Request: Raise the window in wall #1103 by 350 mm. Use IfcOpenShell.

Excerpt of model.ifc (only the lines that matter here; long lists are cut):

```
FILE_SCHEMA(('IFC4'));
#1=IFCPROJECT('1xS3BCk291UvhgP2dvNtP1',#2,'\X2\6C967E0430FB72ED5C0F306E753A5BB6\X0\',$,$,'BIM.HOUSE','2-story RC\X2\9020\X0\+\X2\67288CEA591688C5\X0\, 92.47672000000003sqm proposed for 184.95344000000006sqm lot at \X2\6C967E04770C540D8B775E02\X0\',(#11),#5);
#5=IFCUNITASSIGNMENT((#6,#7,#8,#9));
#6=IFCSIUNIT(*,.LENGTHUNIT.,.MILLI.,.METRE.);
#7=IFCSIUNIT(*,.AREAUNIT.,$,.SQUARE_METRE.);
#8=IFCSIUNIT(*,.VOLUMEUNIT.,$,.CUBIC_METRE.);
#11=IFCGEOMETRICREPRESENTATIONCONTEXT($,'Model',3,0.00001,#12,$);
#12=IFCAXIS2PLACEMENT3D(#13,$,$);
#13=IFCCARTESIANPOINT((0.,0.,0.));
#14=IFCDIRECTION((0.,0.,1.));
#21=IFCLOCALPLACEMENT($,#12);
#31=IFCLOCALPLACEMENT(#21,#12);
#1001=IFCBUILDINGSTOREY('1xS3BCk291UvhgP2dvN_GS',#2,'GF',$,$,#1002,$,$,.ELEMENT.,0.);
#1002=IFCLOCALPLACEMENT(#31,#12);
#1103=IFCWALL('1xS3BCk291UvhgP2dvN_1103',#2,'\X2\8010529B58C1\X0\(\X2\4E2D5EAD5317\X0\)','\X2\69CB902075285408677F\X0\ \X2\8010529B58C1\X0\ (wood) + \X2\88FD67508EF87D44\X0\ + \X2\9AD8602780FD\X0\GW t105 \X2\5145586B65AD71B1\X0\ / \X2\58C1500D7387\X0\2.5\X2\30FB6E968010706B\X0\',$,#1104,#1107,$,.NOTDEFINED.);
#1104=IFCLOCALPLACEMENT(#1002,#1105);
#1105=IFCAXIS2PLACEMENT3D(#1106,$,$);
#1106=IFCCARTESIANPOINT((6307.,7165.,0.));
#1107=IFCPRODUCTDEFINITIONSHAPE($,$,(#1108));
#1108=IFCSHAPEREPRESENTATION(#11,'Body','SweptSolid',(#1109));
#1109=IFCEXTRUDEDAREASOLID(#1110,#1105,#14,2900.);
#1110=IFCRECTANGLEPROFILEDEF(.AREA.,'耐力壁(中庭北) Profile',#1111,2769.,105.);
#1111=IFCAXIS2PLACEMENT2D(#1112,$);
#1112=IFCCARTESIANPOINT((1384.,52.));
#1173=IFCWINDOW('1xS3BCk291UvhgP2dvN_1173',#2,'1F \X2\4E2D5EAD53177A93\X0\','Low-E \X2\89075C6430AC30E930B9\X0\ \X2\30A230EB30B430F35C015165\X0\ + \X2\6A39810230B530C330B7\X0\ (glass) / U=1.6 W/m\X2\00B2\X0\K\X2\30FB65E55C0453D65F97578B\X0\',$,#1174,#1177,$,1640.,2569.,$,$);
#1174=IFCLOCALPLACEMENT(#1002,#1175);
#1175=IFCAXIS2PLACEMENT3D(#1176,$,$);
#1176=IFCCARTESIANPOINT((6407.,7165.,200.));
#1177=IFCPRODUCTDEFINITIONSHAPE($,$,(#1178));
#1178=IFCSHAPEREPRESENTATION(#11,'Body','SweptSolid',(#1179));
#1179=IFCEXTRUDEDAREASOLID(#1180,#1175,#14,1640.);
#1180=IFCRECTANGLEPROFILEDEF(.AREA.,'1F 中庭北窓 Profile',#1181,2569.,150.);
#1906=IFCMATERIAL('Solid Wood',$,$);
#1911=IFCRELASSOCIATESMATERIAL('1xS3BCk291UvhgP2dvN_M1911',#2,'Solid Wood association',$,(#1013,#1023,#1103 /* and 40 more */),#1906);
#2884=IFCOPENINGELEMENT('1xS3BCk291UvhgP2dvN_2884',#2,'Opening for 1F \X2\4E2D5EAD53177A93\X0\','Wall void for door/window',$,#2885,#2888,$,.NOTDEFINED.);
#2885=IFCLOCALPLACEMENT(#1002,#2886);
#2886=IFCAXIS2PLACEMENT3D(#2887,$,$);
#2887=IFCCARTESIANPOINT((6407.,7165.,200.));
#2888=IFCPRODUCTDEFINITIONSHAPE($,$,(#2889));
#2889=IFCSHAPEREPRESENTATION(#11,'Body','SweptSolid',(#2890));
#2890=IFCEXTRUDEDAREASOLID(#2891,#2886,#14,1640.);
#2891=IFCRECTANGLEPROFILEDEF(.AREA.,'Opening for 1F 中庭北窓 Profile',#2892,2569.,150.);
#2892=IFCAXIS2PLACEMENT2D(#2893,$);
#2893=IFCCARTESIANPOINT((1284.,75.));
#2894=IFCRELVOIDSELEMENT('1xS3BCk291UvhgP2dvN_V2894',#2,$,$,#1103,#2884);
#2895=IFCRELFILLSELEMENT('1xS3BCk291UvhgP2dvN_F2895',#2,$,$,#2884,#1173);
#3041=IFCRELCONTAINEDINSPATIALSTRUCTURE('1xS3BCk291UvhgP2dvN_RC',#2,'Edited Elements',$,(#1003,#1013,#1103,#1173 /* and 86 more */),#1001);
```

```python
import numpy as np
import ifcopenshell
import ifcopenshell.api.geometry
import ifcopenshell.util.placement
import ifcopenshell.util.unit

model = ifcopenshell.open("model.ifc")
unit_scale = ifcopenshell.util.unit.calculate_unit_scale(model)

window = model.by_guid("1xS3BCk291UvhgP2dvN_1173")
opening = window.FillsVoids[0].RelatingOpeningElement
dz = 0.35 / unit_scale

shift = np.array([0.0, 0.0, dz])
# The window is not placed relative to its opening, so move both.
for product in (opening, window):
    matrix = ifcopenshell.util.placement.get_local_placement(product.ObjectPlacement)
    matrix[:3, 3] += shift
    ifcopenshell.api.geometry.edit_object_placement(model, product=product, matrix=matrix, is_si=False)

print(f"moved by {dz * unit_scale:+.3f} m")

model.write("model_v2.ifc")
```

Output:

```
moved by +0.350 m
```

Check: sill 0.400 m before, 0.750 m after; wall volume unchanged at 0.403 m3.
